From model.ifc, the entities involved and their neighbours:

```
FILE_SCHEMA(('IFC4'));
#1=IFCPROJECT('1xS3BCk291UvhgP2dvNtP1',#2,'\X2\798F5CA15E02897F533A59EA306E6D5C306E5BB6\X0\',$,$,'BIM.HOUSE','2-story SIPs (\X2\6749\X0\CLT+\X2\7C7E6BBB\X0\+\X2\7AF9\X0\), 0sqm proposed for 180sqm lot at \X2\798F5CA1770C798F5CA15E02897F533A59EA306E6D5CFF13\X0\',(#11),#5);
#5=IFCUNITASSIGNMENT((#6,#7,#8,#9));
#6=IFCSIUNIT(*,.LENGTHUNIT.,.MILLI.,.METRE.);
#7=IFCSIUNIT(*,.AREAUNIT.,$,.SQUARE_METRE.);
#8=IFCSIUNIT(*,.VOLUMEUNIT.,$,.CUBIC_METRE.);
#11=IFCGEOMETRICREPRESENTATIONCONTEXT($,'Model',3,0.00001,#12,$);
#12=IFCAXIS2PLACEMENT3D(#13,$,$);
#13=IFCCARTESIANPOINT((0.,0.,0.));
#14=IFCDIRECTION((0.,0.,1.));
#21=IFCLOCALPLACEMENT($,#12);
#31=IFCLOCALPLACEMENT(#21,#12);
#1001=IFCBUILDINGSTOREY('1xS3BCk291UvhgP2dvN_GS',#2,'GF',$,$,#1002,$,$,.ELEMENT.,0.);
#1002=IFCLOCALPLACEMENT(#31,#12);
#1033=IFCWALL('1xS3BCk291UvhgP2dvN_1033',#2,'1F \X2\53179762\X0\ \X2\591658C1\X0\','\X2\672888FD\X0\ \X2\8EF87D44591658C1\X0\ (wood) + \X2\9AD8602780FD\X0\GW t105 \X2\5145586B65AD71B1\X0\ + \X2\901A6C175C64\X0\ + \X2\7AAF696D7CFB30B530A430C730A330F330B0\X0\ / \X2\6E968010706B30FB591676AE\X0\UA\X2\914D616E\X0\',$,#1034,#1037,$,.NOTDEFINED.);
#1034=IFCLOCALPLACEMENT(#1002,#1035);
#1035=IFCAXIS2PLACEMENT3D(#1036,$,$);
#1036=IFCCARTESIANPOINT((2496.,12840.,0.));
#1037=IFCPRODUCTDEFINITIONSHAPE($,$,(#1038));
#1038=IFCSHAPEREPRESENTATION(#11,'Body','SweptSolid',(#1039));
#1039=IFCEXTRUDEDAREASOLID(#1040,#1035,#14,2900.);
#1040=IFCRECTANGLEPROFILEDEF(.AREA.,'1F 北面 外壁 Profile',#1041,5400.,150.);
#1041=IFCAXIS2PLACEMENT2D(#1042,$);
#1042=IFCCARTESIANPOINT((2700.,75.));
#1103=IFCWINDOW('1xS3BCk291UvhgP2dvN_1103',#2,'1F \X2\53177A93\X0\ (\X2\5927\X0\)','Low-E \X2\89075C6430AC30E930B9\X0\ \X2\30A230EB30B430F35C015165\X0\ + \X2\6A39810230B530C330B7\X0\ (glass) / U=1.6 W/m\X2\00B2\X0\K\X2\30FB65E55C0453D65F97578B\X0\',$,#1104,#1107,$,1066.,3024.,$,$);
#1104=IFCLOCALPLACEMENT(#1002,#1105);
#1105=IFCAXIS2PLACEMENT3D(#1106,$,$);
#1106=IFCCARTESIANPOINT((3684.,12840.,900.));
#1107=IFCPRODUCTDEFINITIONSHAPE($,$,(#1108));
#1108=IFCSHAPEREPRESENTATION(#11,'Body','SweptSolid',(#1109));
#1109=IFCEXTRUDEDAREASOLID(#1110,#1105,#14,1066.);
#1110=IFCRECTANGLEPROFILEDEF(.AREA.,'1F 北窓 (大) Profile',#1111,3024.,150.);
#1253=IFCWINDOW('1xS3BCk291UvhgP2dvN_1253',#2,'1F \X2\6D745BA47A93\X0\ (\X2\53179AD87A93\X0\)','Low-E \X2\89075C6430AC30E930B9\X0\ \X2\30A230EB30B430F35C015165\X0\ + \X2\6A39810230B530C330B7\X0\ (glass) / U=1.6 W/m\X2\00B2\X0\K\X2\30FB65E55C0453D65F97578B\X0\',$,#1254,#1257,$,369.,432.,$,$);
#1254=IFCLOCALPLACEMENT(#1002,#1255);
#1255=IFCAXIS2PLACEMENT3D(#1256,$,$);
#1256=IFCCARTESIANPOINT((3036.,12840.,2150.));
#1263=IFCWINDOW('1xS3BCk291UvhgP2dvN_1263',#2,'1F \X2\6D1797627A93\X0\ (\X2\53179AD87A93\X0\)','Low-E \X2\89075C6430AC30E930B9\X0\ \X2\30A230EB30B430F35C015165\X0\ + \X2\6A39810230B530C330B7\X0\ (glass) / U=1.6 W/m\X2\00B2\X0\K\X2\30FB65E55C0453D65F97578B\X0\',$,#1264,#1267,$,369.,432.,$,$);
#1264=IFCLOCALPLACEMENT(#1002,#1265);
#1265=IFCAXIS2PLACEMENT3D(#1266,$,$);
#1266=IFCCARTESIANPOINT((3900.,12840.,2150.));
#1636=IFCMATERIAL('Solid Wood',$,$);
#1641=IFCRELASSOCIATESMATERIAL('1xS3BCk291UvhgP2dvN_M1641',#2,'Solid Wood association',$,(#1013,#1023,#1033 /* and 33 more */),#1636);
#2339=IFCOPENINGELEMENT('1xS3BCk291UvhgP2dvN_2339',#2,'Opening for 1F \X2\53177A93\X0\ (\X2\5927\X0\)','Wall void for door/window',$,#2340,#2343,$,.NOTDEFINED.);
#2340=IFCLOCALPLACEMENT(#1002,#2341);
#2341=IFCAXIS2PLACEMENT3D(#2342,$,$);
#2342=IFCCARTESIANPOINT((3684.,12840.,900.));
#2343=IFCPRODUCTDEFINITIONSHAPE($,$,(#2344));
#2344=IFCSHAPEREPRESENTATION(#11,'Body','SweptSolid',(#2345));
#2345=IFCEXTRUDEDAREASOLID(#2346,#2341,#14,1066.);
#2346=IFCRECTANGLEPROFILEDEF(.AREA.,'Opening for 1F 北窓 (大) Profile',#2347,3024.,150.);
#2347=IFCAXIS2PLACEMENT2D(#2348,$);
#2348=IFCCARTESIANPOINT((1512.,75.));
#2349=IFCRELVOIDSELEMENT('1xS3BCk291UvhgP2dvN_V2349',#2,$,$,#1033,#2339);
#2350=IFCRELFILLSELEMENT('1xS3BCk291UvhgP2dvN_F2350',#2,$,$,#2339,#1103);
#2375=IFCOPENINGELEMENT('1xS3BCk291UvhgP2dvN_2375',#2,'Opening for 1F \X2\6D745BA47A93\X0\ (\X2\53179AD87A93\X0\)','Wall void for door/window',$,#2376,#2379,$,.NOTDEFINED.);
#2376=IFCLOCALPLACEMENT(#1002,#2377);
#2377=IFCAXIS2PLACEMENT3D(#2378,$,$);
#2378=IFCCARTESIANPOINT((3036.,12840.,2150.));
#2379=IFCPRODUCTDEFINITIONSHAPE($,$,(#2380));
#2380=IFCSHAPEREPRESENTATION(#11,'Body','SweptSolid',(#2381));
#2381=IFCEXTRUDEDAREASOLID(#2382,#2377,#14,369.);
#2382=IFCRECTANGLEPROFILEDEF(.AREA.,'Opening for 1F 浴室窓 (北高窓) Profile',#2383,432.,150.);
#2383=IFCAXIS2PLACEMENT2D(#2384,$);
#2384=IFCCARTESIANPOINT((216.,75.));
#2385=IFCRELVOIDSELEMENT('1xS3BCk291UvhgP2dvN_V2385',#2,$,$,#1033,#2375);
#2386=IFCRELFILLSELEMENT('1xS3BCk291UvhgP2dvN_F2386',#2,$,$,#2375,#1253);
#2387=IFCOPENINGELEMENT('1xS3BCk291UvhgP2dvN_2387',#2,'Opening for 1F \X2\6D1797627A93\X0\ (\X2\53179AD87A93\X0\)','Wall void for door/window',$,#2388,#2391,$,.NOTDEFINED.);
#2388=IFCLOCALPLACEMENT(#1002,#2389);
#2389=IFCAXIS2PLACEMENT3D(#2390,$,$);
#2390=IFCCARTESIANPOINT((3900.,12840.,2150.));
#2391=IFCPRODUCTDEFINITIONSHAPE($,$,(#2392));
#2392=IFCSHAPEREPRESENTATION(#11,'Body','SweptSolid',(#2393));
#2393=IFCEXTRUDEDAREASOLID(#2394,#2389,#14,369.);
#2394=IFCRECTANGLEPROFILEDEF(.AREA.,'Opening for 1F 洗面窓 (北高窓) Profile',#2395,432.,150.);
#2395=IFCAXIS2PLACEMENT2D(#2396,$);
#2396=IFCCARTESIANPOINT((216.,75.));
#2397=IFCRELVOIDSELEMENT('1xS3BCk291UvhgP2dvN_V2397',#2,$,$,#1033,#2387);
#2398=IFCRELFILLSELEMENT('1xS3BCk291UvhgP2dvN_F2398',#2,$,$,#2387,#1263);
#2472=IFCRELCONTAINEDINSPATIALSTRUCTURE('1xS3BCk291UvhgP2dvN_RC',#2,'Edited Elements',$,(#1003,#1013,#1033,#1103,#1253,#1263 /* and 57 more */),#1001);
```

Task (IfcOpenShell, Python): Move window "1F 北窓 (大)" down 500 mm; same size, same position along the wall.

```python
import numpy as np
import ifcopenshell
import ifcopenshell.api.geometry
import ifcopenshell.util.placement
import ifcopenshell.util.unit

model = ifcopenshell.open("model.ifc")
unit_scale = ifcopenshell.util.unit.calculate_unit_scale(model)

window = model.by_guid("1xS3BCk291UvhgP2dvN_1103")
opening = window.FillsVoids[0].RelatingOpeningElement
dz = -0.5 / unit_scale

shift = np.array([0.0, 0.0, dz])
# The window is not placed relative to its opening, so move both.
for product in (opening, window):
    matrix = ifcopenshell.util.placement.get_local_placement(product.ObjectPlacement)
    matrix[:3, 3] += shift
    ifcopenshell.api.geometry.edit_object_placement(model, product=product, matrix=matrix, is_si=False)

print(f"moved by {dz * unit_scale:+.3f} m")

model.write("model_edited.ifc")
```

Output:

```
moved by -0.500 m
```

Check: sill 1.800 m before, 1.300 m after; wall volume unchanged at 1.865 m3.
